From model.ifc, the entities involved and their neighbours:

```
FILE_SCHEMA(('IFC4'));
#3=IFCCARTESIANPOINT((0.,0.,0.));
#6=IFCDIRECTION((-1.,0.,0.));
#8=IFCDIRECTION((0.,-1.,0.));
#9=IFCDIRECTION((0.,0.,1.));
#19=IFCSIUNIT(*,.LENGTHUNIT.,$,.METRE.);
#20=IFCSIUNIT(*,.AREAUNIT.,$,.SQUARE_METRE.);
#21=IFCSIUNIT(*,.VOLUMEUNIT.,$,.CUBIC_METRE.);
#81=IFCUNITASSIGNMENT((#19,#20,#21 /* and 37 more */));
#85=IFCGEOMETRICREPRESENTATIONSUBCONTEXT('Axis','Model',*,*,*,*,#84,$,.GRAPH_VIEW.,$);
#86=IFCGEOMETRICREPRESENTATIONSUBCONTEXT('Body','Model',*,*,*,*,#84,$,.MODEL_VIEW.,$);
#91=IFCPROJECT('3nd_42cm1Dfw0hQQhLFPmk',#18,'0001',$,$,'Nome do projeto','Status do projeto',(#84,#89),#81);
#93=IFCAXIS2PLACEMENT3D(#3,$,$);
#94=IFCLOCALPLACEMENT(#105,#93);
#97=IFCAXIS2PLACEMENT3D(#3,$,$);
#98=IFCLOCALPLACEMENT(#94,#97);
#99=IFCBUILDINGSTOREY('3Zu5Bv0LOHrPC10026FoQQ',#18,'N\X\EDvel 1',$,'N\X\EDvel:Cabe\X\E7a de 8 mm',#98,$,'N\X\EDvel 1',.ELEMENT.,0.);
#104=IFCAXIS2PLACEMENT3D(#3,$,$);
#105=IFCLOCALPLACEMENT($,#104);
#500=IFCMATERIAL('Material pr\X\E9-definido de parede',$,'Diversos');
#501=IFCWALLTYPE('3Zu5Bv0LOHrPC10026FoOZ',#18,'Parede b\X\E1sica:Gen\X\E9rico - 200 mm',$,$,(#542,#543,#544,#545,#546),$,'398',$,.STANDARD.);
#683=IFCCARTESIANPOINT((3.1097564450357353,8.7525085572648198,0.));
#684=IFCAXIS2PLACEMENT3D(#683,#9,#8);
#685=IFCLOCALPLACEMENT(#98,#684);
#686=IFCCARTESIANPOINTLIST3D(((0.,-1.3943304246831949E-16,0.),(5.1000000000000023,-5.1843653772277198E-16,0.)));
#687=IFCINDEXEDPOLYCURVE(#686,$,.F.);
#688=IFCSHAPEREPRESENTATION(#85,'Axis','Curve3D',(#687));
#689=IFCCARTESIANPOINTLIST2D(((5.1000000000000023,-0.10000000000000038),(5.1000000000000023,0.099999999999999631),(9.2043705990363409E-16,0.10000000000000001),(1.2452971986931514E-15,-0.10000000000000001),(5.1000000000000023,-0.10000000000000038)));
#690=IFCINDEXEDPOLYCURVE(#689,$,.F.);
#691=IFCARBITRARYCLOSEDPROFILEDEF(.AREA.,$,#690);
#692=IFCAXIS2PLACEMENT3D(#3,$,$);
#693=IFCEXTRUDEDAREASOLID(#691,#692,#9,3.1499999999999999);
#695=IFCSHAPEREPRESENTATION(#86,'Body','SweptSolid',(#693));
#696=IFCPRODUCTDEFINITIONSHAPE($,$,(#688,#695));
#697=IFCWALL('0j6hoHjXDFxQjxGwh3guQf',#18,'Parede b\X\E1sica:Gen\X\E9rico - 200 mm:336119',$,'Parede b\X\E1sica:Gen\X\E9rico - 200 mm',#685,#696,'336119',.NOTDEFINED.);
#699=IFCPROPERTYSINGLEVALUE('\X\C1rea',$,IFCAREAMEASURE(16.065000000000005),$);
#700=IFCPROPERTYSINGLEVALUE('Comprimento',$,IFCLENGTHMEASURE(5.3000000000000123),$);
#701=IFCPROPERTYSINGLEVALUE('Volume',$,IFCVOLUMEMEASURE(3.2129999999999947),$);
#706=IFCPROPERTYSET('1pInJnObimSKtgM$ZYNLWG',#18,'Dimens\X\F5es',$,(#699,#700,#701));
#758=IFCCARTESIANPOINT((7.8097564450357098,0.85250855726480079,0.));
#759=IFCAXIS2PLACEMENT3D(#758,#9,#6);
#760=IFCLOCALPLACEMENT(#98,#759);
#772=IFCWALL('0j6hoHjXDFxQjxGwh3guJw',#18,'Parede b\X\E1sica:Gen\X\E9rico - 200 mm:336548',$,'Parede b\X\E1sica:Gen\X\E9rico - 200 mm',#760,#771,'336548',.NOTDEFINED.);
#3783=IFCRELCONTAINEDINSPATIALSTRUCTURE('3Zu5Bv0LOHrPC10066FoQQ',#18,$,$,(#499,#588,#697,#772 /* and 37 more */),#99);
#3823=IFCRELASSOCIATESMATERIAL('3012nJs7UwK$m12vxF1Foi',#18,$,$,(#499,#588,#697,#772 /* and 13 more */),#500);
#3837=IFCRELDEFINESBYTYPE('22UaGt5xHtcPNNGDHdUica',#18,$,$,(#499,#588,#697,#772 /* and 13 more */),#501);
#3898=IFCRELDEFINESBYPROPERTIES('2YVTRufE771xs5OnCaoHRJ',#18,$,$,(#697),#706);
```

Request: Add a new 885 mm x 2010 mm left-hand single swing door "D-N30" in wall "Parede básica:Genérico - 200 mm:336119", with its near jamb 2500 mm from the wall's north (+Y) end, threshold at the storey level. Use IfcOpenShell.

```python
import numpy as np
import ifcopenshell
import ifcopenshell.api.feature
import ifcopenshell.api.geometry
import ifcopenshell.api.pset
import ifcopenshell.api.root
import ifcopenshell.api.spatial
import ifcopenshell.geom
import ifcopenshell.util.element
import ifcopenshell.util.placement
import ifcopenshell.util.representation
import ifcopenshell.util.shape
import ifcopenshell.util.unit

model = ifcopenshell.open("model.ifc")
unit_scale = ifcopenshell.util.unit.calculate_unit_scale(model)
area_scale = ifcopenshell.util.unit.calculate_unit_scale(model, "AREAUNIT")
volume_scale = ifcopenshell.util.unit.calculate_unit_scale(model, "VOLUMEUNIT")
settings = ifcopenshell.geom.settings()


def volume(element):
    """Net volume in cubic metres, openings subtracted."""
    shape = ifcopenshell.geom.create_shape(settings, element)
    return ifcopenshell.util.shape.get_volume(shape.geometry)


wall = model.by_guid("0j6hoHjXDFxQjxGwh3guQf")
storey = ifcopenshell.util.element.get_container(wall, ifc_class="IfcBuildingStorey")
context = ifcopenshell.util.representation.get_context(model, "Model", "Body", "MODEL_VIEW")
before = volume(wall)

width, height, from_end, sill = 0.885, 2.01, 2.5, 0.0  # metres

# The wall runs along its own X axis, and the end named is its -X end.
wall_shape = ifcopenshell.geom.create_shape(settings, wall)
x, y, z = ifcopenshell.util.shape.get_vertices(wall_shape.geometry).T
start = x.min() + from_end
face, thickness = float(y.min()), float(y.max() - y.min())
wall_matrix = ifcopenshell.util.placement.get_local_placement(wall.ObjectPlacement)
level = ifcopenshell.util.placement.get_local_placement(storey.ObjectPlacement)[2, 3]


def in_wall(x, y):
    """Placement at x, y metres in the wall's axes, at sill height."""
    matrix = wall_matrix.copy()
    matrix[:, 3] = wall_matrix @ np.array([x / unit_scale, y / unit_scale, 0.0, 1.0])
    matrix[2, 3] = level + sill / unit_scale
    return matrix


# Opening: a box that overshoots both wall faces by 50 mm.
opening = ifcopenshell.api.root.create_entity(model, ifc_class="IfcOpeningElement", predefined_type="OPENING")
box = ifcopenshell.api.geometry.add_wall_representation(
    model, context=context, length=width, height=height, thickness=thickness + 0.1
)
ifcopenshell.api.geometry.assign_representation(model, product=opening, representation=box)
ifcopenshell.api.geometry.edit_object_placement(model, product=opening, matrix=in_wall(start, face - 0.05), is_si=False)
ifcopenshell.api.feature.add_feature(model, feature=opening, element=wall)

door = ifcopenshell.api.root.create_entity(model, ifc_class="IfcDoor", name="D-N30", predefined_type="DOOR")
door.OverallWidth, door.OverallHeight = width / unit_scale, height / unit_scale
door.OperationType = "SINGLE_SWING_LEFT"
body = ifcopenshell.api.geometry.add_door_representation(
    model,
    context=context,
    overall_width=door.OverallWidth,
    overall_height=door.OverallHeight,
    operation_type="SINGLE_SWING_LEFT",
    lining_properties={"LiningDepth": thickness / unit_scale, "ThresholdDepth": thickness / unit_scale},
)
ifcopenshell.api.geometry.assign_representation(model, product=door, representation=body)
ifcopenshell.api.spatial.assign_container(model, products=[door], relating_structure=storey)
ifcopenshell.api.feature.add_filling(model, opening=opening, element=door)

# The lining spans the wall, so the door starts at the wall face.
ifcopenshell.api.geometry.edit_object_placement(model, product=door, matrix=in_wall(start, face), is_si=False)

after = volume(wall)

# Update the wall's stored quantities.
pset = model.by_id(ifcopenshell.util.element.get_pset(wall, "Dimensões", should_inherit=False)["id"])
ifcopenshell.api.pset.edit_pset(model, pset=pset, properties={
    "Área": model.create_entity("IfcAreaMeasure", after / thickness / area_scale),
    "Volume": model.create_entity("IfcVolumeMeasure", after / volume_scale),
})

print(f"wall volume {before:.3f} -> {after:.3f} m3")

model.write("model_edited.ifc")
```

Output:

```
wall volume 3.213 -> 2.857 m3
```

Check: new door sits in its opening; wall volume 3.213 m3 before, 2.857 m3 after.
